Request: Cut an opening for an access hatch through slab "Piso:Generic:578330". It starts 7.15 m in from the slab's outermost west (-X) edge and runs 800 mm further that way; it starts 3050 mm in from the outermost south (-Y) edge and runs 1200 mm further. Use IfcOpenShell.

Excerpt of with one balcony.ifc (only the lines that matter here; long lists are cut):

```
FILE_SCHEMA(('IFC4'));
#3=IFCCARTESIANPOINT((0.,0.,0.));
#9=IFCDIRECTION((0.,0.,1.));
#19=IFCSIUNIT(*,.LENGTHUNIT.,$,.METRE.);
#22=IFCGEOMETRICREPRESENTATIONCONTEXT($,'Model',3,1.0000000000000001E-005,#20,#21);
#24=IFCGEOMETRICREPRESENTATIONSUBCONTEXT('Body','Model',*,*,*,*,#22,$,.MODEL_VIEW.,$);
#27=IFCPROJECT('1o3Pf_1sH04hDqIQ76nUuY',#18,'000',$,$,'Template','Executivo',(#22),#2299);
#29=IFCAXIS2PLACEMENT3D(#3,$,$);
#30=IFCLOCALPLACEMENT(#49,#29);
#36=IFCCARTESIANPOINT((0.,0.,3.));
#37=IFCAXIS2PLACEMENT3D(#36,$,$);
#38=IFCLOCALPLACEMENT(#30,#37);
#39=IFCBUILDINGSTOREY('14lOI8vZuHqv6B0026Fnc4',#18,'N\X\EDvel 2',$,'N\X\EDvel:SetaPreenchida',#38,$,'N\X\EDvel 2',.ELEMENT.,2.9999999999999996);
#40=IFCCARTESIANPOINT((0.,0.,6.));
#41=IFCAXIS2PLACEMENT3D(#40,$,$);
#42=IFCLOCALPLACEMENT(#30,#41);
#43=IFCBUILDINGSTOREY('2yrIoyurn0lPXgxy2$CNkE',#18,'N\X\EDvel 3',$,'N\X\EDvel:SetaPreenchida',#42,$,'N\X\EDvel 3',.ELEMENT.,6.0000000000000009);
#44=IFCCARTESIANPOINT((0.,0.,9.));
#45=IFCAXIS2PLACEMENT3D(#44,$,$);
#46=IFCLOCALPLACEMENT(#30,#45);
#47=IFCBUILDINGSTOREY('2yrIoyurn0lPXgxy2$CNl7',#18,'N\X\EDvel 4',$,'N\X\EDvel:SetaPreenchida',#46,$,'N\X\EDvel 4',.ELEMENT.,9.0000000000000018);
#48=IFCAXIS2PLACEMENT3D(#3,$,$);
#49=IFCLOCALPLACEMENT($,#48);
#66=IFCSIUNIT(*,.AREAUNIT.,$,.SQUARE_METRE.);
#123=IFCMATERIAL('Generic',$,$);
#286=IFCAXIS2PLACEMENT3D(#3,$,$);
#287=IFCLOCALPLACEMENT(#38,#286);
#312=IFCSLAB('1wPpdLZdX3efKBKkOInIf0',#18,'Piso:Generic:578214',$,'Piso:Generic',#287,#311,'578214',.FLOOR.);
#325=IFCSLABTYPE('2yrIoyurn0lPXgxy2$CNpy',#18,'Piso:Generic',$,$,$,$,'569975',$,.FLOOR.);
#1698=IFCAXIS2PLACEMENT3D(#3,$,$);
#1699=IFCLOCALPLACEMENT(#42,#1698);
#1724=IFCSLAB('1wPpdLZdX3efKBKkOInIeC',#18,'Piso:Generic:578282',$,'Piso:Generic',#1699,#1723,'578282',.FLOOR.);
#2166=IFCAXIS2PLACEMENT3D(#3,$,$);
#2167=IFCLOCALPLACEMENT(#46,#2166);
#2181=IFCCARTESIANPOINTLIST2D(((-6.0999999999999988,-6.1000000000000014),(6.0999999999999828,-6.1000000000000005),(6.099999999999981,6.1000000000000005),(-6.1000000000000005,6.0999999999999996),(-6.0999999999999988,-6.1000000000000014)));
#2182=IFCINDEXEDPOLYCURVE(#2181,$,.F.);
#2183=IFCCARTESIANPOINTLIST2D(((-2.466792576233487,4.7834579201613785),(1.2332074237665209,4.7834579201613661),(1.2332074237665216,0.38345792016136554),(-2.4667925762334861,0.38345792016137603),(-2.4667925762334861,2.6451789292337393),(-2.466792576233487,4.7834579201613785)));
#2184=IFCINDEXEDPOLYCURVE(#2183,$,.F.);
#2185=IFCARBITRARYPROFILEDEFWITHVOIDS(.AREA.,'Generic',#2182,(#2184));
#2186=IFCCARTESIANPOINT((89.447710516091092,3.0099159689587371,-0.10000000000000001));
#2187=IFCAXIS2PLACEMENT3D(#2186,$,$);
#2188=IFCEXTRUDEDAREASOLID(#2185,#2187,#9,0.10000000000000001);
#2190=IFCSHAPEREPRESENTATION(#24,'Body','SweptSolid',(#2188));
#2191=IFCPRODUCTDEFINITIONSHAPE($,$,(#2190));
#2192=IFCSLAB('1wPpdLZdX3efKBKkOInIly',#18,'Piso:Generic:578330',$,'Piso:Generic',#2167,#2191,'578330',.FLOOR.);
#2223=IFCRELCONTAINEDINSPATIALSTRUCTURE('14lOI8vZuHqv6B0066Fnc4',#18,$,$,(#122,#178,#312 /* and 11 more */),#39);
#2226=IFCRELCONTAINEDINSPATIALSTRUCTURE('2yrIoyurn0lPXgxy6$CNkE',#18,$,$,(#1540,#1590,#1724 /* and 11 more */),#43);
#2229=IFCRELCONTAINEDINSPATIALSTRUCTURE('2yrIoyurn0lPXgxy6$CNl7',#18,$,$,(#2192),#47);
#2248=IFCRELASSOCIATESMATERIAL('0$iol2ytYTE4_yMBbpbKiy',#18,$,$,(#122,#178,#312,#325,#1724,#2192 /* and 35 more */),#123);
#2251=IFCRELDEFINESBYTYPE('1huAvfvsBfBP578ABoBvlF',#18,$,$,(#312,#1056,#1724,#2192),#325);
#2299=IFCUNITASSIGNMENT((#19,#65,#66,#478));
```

```python
import numpy as np
import ifcopenshell
import ifcopenshell.api.feature
import ifcopenshell.api.geometry
import ifcopenshell.api.root
import ifcopenshell.geom
import ifcopenshell.util.placement
import ifcopenshell.util.representation
import ifcopenshell.util.shape
import ifcopenshell.util.unit

model = ifcopenshell.open("with one balcony.ifc")
unit_scale = ifcopenshell.util.unit.calculate_unit_scale(model)
settings = ifcopenshell.geom.settings()


def volume(element):
    """Net volume in cubic metres, openings subtracted."""
    shape = ifcopenshell.geom.create_shape(settings, element)
    return ifcopenshell.util.shape.get_volume(shape.geometry)


slab = model.by_id(2192)
before = volume(slab)

# Extent in the slab's own axes, in metres. The edges named are its -X and -Y sides.
slab_shape = ifcopenshell.geom.create_shape(settings, slab)
vertices = ifcopenshell.util.shape.get_vertices(slab_shape.geometry)
x_min, y_min, bottom = vertices.min(axis=0)
top = vertices[:, 2].max()

opening = ifcopenshell.api.root.create_entity(model, ifc_class="IfcOpeningElement", name="Access hatch opening", predefined_type="OPENING")
context = ifcopenshell.util.representation.get_context(model, "Model", "Body", "MODEL_VIEW")
width, depth = 0.8, 1.2
outline = [(0.0, 0.0), (width, 0.0), (width, depth), (0.0, depth), (0.0, 0.0)]
# Overshoot both faces by 50 mm so the cut is clean.
shape = ifcopenshell.api.geometry.add_slab_representation(
    model, context=context, depth=top - bottom + 0.1, polyline=outline
)
ifcopenshell.api.geometry.assign_representation(model, product=opening, representation=shape)

matrix = ifcopenshell.util.placement.get_local_placement(slab.ObjectPlacement)
matrix[:, 3] = matrix @ np.append(np.array([x_min + 7.15, y_min + 3.05, bottom - 0.05]) / unit_scale, 1.0)
ifcopenshell.api.geometry.edit_object_placement(model, product=opening, matrix=matrix, is_si=False)
ifcopenshell.api.feature.add_feature(model, feature=opening, element=slab)

after = volume(slab)

print(f"slab volume {before:.3f} -> {after:.3f} m3")

model.write("with one balcony_rev.ifc")
```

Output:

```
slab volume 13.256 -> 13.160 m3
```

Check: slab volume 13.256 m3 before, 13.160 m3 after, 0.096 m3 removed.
